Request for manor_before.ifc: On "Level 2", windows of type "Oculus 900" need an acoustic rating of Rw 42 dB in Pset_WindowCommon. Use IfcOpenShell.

First a look at what the model holds.

```python
import ifcopenshell
import ifcopenshell.util.element

model = ifcopenshell.open("manor_before.ifc")
print(model.schema)
storey = next(s for s in model.by_type("IfcBuildingStorey") if s.Name == "Level 2")
windows = [e for e in ifcopenshell.util.element.get_decomposition(storey) if e.is_a("IfcWindow")]
seen = {}
for e in windows:
    element_type = ifcopenshell.util.element.get_type(e)
    key = (element_type.Name if element_type != e and element_type else None, ifcopenshell.util.element.get_pset(e, "Pset_WindowCommon", "AcousticRating"))
    seen[key] = seen.get(key, 0) + 1
for (name, value), count in sorted(seen.items(), key=str):
    print(count, "x", name, "|", value)
```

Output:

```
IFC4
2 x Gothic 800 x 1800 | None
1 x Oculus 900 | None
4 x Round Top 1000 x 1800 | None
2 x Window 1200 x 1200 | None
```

```python
import ifcopenshell
import ifcopenshell.api.pset
import ifcopenshell.util.element

model = ifcopenshell.open("manor_before.ifc")

storey = next(s for s in model.by_type("IfcBuildingStorey") if s.Name == "Level 2")
windows = [e for e in ifcopenshell.util.element.get_decomposition(storey) if e.is_a("IfcWindow")]

count = 0
for e in windows:
    element_type = ifcopenshell.util.element.get_type(e)
    if element_type in (None, e) or element_type.Name != "Oculus 900":
        continue
    # add_pset returns the element's existing set when there is one.
    pset = ifcopenshell.api.pset.add_pset(model, product=e, name="Pset_WindowCommon")
    ifcopenshell.api.pset.edit_pset(model, pset=pset, properties={"AcousticRating": "Rw 42 dB"})
    count += 1

print(count, "windows updated")

model.write("manor_before_updated.ifc")
```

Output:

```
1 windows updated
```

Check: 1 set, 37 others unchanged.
